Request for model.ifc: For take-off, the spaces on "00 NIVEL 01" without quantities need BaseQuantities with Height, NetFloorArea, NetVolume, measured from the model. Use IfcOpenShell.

First a look at what the model holds.

```python
import ifcopenshell
import ifcopenshell.util.element
import ifcopenshell.util.unit

model = ifcopenshell.open("model.ifc")
print(model.schema)
for unit_type in ("LENGTHUNIT", "AREAUNIT", "VOLUMEUNIT"):
    print(unit_type, ifcopenshell.util.unit.calculate_unit_scale(model, unit_type))
storey = next(s for s in model.by_type("IfcBuildingStorey") if s.Name == "00 NIVEL 01")
spaces = [e for e in ifcopenshell.util.element.get_decomposition(storey) if e.is_a("IfcSpace")]
for e in sorted(spaces, key=lambda e: e.id()):
    print(e.id(), e.is_a(), e.Name, list(ifcopenshell.util.element.get_psets(e, qtos_only=True)), sep=" | ")
```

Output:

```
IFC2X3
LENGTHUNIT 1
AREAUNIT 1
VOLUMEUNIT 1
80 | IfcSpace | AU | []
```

```python
import ifcopenshell
import ifcopenshell.api.pset
import ifcopenshell.geom
import ifcopenshell.util.element
import ifcopenshell.util.shape
import ifcopenshell.util.unit

model = ifcopenshell.open("model.ifc")
unit_scale = ifcopenshell.util.unit.calculate_unit_scale(model)
area_scale = ifcopenshell.util.unit.calculate_unit_scale(model, "AREAUNIT")
volume_scale = ifcopenshell.util.unit.calculate_unit_scale(model, "VOLUMEUNIT")
settings = ifcopenshell.geom.settings()

storey = next(s for s in model.by_type("IfcBuildingStorey") if s.Name == "00 NIVEL 01")
spaces = [e for e in ifcopenshell.util.element.get_decomposition(storey) if e.is_a("IfcSpace")]

for e in sorted(spaces, key=lambda e: e.id()):
    if ifcopenshell.util.element.get_psets(e, qtos_only=True, should_inherit=False):
        continue
    # Geometry comes back in metres, in the element's own axes.
    shape = ifcopenshell.geom.create_shape(settings, e)
    values = {
        "Height": ifcopenshell.util.shape.get_z(shape.geometry) / unit_scale,
        "NetFloorArea": ifcopenshell.util.shape.get_footprint_area(shape.geometry) / area_scale,
        "NetVolume": ifcopenshell.util.shape.get_volume(shape.geometry) / volume_scale,
    }
    qto = ifcopenshell.api.pset.add_qto(model, product=e, name="BaseQuantities")
    ifcopenshell.api.pset.edit_qto(model, qto=qto, properties=values)
    print(e.id(), {k: round(v, 3) for k, v in values.items()})

model.write("model_rev.ifc")
```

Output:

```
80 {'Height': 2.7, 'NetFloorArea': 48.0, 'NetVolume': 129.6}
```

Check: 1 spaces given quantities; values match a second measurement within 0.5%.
